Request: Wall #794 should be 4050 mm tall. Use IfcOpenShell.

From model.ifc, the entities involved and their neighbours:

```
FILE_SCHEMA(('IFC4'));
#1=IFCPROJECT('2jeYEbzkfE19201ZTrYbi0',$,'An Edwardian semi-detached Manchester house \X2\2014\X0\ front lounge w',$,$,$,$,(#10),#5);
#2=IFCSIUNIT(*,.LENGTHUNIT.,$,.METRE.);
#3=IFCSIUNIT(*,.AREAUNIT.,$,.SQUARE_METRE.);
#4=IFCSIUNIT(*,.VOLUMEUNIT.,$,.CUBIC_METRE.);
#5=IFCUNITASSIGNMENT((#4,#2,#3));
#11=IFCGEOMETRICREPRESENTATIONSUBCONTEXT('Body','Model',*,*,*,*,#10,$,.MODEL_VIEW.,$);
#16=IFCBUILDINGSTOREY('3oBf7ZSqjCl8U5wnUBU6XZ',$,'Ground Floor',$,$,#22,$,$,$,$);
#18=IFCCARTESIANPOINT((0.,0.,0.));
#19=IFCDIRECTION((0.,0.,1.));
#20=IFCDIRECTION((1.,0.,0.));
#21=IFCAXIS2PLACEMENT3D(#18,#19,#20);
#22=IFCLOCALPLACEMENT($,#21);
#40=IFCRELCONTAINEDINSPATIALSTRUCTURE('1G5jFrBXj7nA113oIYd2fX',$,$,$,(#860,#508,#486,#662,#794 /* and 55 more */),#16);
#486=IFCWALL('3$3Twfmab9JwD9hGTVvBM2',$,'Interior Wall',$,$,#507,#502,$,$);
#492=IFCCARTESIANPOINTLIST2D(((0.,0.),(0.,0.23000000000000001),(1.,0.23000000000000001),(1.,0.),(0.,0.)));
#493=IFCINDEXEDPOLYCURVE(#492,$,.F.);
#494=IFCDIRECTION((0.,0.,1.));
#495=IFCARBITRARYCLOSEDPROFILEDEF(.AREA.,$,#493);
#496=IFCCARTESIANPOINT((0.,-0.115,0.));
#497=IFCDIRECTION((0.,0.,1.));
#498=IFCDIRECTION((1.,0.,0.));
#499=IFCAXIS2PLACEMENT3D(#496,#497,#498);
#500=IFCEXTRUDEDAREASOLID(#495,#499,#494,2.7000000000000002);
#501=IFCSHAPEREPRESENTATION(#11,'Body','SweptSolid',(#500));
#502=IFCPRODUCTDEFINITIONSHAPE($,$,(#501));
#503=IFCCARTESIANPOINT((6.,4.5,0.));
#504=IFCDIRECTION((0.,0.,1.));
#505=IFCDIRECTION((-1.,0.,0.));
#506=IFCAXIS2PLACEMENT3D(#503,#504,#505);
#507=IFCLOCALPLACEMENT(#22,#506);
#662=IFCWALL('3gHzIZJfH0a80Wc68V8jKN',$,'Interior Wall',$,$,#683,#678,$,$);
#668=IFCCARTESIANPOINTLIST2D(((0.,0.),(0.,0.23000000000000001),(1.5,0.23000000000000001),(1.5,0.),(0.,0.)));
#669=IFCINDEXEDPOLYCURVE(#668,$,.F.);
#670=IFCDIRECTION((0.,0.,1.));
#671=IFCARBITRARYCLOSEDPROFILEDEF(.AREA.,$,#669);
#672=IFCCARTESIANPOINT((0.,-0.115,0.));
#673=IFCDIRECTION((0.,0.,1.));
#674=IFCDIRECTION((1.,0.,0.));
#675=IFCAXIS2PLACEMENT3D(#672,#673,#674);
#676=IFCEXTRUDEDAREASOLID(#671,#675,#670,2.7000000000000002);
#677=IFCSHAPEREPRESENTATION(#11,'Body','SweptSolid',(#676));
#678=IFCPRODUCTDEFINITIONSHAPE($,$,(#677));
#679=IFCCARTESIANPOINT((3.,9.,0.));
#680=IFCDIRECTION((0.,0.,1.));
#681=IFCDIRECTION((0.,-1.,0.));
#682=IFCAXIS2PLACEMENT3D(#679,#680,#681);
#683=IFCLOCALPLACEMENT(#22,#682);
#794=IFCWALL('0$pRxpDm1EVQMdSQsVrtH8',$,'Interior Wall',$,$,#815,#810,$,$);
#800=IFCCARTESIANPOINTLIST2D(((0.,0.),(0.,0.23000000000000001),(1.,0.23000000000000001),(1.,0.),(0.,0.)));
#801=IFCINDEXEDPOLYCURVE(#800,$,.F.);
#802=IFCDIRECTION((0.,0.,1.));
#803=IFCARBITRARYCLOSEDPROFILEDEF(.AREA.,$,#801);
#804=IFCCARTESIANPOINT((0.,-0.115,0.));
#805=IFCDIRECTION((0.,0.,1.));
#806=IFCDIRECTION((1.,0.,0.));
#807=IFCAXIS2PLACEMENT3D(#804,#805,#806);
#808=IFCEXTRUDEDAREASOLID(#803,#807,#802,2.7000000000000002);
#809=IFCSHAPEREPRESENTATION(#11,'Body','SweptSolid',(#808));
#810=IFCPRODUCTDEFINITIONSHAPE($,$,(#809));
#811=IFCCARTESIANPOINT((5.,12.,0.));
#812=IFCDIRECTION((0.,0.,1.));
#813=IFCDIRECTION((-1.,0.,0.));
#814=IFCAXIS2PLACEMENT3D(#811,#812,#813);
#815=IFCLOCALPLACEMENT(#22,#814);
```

```python
import ifcopenshell
import ifcopenshell.geom
import ifcopenshell.util.representation
import ifcopenshell.util.shape
import ifcopenshell.util.unit

model = ifcopenshell.open("model.ifc")
unit_scale = ifcopenshell.util.unit.calculate_unit_scale(model)
settings = ifcopenshell.geom.settings()


def volume(element):
    """Net volume in cubic metres, openings subtracted."""
    shape = ifcopenshell.geom.create_shape(settings, element)
    return ifcopenshell.util.shape.get_volume(shape.geometry)


wall = model.by_guid("0$pRxpDm1EVQMdSQsVrtH8")
before = volume(wall)

body = ifcopenshell.util.representation.get_representation(wall, "Model", "Body")
solid = body.Items[0]
old_height = solid.Depth
solid.Depth = 4.05 / unit_scale
after = volume(wall)

print(f"height {old_height:g} -> {solid.Depth:g}, volume {before:.3f} -> {after:.3f} m3")

model.write("model_edited.ifc")
```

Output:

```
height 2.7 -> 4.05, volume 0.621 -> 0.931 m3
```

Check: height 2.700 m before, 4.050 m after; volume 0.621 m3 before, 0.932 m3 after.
